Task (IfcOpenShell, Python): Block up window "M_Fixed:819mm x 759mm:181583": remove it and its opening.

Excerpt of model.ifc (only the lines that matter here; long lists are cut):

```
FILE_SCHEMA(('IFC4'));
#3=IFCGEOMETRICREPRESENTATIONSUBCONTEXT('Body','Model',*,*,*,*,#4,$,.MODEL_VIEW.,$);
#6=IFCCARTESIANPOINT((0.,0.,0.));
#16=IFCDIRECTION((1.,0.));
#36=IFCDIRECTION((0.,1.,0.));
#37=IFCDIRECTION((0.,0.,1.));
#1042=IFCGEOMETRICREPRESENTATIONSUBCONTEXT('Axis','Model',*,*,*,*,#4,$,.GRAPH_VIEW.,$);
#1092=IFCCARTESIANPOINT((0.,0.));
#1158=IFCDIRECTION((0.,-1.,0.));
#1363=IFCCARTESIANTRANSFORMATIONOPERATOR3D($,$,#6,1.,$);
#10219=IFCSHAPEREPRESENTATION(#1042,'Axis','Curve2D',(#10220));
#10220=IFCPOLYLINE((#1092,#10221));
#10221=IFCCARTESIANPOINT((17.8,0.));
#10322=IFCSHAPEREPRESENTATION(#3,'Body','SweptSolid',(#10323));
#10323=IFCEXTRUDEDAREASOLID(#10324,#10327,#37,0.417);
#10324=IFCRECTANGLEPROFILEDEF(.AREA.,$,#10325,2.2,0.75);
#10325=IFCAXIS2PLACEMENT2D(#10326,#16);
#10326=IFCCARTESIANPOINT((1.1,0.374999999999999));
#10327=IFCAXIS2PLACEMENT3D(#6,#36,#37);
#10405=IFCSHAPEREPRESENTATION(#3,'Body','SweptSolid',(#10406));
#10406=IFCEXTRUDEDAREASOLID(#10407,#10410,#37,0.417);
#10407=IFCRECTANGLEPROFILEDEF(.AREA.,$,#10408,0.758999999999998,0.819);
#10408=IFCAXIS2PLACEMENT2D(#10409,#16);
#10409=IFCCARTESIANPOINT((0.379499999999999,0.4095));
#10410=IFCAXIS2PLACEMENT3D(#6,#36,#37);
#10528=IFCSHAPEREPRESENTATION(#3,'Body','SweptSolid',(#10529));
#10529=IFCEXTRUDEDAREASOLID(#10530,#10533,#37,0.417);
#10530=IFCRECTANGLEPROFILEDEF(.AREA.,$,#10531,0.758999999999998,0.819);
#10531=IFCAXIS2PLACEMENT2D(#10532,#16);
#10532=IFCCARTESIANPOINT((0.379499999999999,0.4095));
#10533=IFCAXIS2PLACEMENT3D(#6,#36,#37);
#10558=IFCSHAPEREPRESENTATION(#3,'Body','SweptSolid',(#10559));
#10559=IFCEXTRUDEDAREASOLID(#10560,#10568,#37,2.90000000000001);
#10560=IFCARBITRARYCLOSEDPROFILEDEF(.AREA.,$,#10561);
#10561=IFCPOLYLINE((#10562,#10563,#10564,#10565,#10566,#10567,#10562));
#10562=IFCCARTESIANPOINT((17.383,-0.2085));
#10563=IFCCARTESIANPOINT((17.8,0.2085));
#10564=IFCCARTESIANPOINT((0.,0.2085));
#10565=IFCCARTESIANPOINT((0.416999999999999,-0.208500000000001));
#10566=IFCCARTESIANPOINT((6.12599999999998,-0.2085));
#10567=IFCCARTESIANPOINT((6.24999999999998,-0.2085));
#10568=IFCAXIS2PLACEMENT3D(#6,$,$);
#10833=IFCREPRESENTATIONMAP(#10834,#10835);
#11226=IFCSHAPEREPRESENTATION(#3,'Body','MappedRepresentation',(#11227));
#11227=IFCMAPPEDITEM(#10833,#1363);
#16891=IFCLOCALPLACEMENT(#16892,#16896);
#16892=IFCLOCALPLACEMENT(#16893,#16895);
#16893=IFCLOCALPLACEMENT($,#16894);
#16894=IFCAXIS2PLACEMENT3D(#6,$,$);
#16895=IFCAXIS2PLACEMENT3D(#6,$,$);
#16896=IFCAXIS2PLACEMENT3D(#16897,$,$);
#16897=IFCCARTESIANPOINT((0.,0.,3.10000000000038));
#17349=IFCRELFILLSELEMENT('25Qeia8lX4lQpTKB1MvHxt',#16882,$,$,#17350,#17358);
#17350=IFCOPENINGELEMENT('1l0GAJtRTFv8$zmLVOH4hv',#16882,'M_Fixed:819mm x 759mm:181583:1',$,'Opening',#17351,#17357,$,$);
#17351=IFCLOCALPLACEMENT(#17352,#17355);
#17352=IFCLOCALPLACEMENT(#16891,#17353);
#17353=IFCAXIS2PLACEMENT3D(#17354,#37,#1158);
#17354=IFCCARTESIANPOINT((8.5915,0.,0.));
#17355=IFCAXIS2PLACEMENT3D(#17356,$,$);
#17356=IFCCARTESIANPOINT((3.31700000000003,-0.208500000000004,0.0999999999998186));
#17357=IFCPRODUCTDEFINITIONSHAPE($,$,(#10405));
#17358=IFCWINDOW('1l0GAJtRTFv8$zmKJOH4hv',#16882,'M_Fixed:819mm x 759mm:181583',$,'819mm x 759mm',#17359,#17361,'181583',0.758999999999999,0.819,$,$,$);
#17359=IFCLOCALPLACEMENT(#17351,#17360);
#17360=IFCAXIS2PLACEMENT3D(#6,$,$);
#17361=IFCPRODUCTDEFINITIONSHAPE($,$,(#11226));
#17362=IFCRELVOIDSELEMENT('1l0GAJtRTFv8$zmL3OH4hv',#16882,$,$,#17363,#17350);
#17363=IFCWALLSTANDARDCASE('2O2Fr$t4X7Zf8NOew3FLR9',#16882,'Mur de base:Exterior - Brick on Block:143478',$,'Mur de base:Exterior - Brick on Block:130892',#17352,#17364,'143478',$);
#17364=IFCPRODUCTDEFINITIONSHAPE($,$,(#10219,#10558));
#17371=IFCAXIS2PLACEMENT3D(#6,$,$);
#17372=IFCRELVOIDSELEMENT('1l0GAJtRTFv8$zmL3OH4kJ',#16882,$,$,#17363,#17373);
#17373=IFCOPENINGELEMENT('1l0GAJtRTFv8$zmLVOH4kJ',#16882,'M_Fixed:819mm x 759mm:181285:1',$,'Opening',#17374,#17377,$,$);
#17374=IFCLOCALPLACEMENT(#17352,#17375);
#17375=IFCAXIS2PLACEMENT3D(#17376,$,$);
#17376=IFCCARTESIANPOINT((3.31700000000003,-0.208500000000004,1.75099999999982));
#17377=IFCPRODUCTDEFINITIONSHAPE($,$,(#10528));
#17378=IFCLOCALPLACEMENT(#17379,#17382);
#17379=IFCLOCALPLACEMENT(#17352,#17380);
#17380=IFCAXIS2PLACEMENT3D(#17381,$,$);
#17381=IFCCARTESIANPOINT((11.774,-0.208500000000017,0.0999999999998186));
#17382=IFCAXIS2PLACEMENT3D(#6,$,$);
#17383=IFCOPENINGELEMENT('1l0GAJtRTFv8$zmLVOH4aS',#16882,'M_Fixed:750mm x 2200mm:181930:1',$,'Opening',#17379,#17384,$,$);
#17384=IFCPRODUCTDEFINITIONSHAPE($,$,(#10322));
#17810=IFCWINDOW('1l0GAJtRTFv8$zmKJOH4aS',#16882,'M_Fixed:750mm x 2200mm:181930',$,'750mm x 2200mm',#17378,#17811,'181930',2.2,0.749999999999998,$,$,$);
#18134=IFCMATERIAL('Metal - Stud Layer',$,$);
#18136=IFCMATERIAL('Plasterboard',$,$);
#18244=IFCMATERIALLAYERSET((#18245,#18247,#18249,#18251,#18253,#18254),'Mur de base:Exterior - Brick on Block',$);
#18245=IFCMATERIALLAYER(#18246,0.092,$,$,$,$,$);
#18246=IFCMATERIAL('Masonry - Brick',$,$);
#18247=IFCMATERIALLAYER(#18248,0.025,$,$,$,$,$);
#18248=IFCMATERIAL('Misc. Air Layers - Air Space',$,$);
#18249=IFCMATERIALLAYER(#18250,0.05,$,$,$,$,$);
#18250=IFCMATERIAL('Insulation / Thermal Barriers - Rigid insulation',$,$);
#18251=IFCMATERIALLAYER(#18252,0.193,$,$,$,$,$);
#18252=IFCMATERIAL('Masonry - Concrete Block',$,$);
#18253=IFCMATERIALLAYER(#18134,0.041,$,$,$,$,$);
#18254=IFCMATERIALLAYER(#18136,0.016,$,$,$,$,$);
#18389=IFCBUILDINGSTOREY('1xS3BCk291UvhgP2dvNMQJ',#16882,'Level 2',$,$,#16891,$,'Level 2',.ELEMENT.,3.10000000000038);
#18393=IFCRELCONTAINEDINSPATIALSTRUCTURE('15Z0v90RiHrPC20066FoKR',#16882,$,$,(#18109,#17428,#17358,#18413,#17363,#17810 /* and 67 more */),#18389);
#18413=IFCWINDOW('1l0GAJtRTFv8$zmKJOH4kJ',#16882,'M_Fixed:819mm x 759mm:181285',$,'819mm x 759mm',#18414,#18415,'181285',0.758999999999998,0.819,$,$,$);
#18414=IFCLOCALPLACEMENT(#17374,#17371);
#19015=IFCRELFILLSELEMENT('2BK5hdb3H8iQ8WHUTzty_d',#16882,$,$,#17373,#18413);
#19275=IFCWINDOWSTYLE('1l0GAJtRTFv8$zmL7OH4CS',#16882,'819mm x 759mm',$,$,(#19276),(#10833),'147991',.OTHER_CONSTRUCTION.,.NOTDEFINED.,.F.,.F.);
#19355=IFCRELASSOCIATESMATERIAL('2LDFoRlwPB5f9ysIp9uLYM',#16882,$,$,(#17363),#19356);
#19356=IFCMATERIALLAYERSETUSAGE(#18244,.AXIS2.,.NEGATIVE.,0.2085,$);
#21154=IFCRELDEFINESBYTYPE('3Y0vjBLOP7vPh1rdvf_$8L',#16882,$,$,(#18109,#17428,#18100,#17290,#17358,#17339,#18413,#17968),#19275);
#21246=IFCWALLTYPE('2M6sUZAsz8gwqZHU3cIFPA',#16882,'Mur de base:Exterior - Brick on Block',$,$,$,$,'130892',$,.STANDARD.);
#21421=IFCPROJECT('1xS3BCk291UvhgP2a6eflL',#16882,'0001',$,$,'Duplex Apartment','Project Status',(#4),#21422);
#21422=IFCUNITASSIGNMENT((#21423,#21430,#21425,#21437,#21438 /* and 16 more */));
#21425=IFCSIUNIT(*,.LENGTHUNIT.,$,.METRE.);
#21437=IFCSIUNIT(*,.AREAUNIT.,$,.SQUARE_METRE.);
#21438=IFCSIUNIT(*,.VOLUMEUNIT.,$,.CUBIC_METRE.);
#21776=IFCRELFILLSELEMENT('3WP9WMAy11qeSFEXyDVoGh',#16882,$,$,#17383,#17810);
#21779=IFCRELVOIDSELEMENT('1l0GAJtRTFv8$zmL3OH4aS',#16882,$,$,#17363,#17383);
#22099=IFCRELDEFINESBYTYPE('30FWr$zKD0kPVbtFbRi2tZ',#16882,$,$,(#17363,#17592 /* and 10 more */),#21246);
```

```python
import ifcopenshell
import ifcopenshell.api.feature
import ifcopenshell.api.root
import ifcopenshell.geom
import ifcopenshell.util.shape

model = ifcopenshell.open("model.ifc")
settings = ifcopenshell.geom.settings()


def volume(element):
    """Net volume in cubic metres, openings subtracted."""
    shape = ifcopenshell.geom.create_shape(settings, element)
    return ifcopenshell.util.shape.get_volume(shape.geometry)


window = model.by_guid("1l0GAJtRTFv8$zmKJOH4hv")
opening = window.FillsVoids[0].RelatingOpeningElement
wall = opening.VoidsElements[0].RelatingBuildingElement
before = volume(wall)

ifcopenshell.api.root.remove_product(model, product=window)
ifcopenshell.api.feature.remove_feature(model, feature=opening)

after = volume(wall)

print(f"wall volume {before:.3f} -> {after:.3f} m3")

model.write("model_updated.ifc")
```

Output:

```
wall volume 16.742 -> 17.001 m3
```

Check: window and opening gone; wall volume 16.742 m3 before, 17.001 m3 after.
